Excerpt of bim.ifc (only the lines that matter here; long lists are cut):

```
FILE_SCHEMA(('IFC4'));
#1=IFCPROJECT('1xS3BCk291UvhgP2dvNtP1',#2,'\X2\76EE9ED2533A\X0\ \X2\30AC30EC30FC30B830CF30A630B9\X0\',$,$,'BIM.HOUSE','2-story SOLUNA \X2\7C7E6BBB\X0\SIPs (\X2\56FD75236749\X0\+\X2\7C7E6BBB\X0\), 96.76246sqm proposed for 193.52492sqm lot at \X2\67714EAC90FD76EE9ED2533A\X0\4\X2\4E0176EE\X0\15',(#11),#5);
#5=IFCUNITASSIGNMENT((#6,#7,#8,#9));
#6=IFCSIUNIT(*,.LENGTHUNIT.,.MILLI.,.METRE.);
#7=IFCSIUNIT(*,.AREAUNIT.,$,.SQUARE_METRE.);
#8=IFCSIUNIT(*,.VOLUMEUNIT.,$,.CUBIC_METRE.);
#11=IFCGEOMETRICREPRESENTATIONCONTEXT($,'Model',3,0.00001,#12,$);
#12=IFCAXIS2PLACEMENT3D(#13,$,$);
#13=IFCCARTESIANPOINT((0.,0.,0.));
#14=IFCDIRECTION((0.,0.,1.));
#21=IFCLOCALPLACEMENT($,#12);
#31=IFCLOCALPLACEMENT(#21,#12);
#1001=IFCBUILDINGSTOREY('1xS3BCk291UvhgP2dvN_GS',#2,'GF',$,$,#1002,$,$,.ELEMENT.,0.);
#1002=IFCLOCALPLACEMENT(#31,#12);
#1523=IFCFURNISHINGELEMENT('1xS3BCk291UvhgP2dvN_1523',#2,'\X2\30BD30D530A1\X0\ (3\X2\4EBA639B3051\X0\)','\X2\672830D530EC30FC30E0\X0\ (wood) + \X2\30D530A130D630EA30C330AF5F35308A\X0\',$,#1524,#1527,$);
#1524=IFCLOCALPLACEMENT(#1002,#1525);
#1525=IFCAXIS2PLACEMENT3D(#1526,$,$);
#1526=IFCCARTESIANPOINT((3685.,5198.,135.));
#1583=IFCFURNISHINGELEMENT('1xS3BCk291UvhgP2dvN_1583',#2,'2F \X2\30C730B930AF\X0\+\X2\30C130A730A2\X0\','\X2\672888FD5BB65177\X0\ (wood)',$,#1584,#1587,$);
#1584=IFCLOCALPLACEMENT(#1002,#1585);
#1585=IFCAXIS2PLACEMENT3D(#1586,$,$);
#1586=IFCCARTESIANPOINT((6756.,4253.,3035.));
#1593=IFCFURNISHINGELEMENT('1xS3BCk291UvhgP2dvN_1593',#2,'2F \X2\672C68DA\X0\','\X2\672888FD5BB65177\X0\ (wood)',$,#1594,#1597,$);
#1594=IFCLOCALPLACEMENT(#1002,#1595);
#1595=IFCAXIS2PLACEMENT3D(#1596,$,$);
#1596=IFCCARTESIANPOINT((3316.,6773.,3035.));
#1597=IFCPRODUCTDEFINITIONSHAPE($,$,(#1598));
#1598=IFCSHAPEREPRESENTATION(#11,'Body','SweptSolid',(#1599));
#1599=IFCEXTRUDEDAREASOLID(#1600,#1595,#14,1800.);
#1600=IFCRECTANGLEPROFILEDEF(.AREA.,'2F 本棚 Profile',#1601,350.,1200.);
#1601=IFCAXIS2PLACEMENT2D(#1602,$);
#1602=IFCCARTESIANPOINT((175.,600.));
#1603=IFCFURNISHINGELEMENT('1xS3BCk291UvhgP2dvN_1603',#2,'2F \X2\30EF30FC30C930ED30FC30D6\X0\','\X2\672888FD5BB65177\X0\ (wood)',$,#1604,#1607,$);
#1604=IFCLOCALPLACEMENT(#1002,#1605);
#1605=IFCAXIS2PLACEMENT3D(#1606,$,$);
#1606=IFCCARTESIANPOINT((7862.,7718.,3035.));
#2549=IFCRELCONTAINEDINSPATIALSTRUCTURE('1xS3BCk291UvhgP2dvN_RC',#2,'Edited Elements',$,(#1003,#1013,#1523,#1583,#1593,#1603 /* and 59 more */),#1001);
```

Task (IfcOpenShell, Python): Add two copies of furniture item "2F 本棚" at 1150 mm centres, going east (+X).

```python
import numpy as np
import ifcopenshell
import ifcopenshell.api.geometry
import ifcopenshell.api.root
import ifcopenshell.util.element
import ifcopenshell.util.placement

model = ifcopenshell.open("bim.ifc")


def reuse_history(source, copy):
    """copy_class also copies each property set's owner history, people and application; keep the originals."""
    for rel in copy.IsDefinedBy:
        if rel.is_a("IfcRelDefinesByProperties") and (history := rel.RelatingPropertyDefinition.OwnerHistory):
            rel.RelatingPropertyDefinition.OwnerHistory = source.OwnerHistory
            ifcopenshell.util.element.remove_deep2(model, history)


source = model.by_id(1593)
base = ifcopenshell.util.placement.get_local_placement(source.ObjectPlacement)
step = np.array([1.0, 0.0, 0.0]) * 1150.0

for i in range(1, 3):
    copy = ifcopenshell.api.root.copy_class(model, product=source)
    copy.Representation = ifcopenshell.util.element.copy_deep(
        model, source.Representation, exclude=["IfcGeometricRepresentationContext", "IfcRepresentationMap"]
    )
    reuse_history(source, copy)
    matrix = base.copy()
    matrix[:3, 3] += i * step
    print("added at", matrix[:3, 3].round(3) + 0.0)
    ifcopenshell.api.geometry.edit_object_placement(model, product=copy, matrix=matrix, is_si=False)

model.write("bim-out.ifc")
```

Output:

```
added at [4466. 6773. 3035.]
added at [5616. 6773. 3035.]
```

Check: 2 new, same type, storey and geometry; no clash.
